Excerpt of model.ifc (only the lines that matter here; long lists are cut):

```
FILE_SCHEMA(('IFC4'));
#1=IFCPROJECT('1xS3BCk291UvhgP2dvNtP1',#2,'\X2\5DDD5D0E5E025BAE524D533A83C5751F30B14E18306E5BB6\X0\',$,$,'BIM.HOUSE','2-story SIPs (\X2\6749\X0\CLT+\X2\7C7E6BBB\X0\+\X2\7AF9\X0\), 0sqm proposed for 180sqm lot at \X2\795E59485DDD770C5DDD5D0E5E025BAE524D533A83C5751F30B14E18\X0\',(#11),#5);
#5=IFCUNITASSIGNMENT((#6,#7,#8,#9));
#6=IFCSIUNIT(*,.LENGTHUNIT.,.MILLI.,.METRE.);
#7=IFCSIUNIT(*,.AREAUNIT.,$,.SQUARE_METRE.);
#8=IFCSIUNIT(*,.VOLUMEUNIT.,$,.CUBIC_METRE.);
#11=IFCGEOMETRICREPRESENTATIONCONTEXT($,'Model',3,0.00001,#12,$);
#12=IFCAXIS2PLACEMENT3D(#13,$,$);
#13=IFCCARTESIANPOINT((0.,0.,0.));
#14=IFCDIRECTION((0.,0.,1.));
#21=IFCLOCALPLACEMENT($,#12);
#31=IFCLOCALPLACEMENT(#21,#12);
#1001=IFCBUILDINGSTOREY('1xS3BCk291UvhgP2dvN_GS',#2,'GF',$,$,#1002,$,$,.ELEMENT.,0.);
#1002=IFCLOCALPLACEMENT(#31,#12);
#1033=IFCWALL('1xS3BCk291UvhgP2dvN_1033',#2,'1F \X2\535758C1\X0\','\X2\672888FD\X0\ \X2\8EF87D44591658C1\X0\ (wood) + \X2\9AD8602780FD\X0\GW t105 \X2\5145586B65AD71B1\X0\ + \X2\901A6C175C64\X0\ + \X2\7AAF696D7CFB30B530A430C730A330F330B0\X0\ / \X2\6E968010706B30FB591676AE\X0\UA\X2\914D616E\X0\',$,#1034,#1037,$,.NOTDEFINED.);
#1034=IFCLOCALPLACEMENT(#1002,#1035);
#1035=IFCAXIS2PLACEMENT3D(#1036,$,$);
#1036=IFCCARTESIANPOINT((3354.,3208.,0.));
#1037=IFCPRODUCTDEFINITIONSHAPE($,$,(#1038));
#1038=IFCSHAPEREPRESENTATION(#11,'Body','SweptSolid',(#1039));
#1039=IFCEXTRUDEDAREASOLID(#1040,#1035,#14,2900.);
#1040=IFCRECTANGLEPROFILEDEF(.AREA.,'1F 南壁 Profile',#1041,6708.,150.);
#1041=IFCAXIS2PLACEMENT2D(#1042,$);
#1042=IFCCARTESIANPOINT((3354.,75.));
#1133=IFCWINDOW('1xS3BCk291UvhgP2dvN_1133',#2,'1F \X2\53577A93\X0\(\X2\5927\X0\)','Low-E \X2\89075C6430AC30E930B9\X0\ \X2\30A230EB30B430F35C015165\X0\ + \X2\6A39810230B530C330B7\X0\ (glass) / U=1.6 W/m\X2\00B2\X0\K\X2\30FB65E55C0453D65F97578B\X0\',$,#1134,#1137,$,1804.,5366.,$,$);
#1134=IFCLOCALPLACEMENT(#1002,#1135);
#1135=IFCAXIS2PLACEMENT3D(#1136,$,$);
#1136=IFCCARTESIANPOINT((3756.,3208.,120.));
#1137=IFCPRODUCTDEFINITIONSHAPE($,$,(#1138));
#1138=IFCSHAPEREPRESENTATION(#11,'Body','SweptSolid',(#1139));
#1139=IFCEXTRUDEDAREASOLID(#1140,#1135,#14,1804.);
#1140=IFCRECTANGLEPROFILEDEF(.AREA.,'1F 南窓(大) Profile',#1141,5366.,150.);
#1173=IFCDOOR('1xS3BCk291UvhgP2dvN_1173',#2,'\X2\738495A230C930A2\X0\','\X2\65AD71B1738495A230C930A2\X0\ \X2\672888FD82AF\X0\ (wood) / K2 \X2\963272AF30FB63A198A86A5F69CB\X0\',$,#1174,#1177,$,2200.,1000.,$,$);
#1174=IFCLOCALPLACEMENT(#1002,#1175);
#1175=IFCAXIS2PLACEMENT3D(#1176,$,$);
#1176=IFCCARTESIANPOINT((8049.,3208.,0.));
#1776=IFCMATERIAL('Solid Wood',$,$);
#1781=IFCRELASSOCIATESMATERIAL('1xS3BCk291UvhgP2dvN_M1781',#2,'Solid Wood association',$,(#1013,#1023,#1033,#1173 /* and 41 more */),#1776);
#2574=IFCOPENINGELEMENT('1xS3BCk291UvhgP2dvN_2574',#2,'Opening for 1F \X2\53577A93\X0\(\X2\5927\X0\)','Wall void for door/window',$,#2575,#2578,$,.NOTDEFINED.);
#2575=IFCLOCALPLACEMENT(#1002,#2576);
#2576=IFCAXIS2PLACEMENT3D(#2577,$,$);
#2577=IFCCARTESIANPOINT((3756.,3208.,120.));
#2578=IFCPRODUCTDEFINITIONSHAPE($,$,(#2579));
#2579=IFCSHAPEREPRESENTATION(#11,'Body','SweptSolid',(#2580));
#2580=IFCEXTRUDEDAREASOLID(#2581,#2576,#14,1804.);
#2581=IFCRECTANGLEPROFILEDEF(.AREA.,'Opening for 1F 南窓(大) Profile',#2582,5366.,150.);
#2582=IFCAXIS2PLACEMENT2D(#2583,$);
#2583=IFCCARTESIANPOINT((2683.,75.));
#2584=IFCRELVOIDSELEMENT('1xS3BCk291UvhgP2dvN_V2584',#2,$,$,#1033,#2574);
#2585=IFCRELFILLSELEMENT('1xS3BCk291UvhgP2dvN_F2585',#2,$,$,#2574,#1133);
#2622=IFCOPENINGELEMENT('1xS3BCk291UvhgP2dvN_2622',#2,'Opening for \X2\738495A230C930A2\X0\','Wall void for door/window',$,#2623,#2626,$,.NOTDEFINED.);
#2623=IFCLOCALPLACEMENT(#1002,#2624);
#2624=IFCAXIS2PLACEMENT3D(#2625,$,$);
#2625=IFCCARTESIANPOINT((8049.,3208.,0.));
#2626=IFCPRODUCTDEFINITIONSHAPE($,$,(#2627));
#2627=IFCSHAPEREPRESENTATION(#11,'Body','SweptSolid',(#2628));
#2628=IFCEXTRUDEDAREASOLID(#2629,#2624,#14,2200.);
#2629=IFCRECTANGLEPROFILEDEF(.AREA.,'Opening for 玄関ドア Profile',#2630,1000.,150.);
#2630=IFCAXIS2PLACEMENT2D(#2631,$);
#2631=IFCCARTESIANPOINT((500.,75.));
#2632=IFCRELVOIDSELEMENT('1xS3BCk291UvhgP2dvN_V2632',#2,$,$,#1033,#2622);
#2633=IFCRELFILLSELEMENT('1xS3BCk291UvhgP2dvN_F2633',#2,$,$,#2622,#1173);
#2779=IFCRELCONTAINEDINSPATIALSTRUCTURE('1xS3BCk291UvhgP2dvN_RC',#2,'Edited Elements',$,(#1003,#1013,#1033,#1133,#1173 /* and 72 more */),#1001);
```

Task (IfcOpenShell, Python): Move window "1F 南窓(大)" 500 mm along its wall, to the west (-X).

```python
import ifcopenshell
import ifcopenshell.api.geometry
import ifcopenshell.util.placement
import ifcopenshell.util.unit

model = ifcopenshell.open("model.ifc")
unit_scale = ifcopenshell.util.unit.calculate_unit_scale(model)

window = model.by_id(1133)
opening = window.FillsVoids[0].RelatingOpeningElement
wall = opening.VoidsElements[0].RelatingBuildingElement

wall_matrix = ifcopenshell.util.placement.get_local_placement(wall.ObjectPlacement)
shift = wall_matrix[:3, 0] * -0.5 / unit_scale
before = ifcopenshell.util.placement.get_local_placement(window.ObjectPlacement)[:3, 3].copy()

# The window is not placed relative to its opening, so move both.
for product in (opening, window):
    matrix = ifcopenshell.util.placement.get_local_placement(product.ObjectPlacement)
    matrix[:3, 3] += shift
    ifcopenshell.api.geometry.edit_object_placement(model, product=product, matrix=matrix, is_si=False)

after = ifcopenshell.util.placement.get_local_placement(window.ObjectPlacement)[:3, 3]
print("window moved by", (after - before).round(3) + 0.0)

model.write("model_rev.ifc")
```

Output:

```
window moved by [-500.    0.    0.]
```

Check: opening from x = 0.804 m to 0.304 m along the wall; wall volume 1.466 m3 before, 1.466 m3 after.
